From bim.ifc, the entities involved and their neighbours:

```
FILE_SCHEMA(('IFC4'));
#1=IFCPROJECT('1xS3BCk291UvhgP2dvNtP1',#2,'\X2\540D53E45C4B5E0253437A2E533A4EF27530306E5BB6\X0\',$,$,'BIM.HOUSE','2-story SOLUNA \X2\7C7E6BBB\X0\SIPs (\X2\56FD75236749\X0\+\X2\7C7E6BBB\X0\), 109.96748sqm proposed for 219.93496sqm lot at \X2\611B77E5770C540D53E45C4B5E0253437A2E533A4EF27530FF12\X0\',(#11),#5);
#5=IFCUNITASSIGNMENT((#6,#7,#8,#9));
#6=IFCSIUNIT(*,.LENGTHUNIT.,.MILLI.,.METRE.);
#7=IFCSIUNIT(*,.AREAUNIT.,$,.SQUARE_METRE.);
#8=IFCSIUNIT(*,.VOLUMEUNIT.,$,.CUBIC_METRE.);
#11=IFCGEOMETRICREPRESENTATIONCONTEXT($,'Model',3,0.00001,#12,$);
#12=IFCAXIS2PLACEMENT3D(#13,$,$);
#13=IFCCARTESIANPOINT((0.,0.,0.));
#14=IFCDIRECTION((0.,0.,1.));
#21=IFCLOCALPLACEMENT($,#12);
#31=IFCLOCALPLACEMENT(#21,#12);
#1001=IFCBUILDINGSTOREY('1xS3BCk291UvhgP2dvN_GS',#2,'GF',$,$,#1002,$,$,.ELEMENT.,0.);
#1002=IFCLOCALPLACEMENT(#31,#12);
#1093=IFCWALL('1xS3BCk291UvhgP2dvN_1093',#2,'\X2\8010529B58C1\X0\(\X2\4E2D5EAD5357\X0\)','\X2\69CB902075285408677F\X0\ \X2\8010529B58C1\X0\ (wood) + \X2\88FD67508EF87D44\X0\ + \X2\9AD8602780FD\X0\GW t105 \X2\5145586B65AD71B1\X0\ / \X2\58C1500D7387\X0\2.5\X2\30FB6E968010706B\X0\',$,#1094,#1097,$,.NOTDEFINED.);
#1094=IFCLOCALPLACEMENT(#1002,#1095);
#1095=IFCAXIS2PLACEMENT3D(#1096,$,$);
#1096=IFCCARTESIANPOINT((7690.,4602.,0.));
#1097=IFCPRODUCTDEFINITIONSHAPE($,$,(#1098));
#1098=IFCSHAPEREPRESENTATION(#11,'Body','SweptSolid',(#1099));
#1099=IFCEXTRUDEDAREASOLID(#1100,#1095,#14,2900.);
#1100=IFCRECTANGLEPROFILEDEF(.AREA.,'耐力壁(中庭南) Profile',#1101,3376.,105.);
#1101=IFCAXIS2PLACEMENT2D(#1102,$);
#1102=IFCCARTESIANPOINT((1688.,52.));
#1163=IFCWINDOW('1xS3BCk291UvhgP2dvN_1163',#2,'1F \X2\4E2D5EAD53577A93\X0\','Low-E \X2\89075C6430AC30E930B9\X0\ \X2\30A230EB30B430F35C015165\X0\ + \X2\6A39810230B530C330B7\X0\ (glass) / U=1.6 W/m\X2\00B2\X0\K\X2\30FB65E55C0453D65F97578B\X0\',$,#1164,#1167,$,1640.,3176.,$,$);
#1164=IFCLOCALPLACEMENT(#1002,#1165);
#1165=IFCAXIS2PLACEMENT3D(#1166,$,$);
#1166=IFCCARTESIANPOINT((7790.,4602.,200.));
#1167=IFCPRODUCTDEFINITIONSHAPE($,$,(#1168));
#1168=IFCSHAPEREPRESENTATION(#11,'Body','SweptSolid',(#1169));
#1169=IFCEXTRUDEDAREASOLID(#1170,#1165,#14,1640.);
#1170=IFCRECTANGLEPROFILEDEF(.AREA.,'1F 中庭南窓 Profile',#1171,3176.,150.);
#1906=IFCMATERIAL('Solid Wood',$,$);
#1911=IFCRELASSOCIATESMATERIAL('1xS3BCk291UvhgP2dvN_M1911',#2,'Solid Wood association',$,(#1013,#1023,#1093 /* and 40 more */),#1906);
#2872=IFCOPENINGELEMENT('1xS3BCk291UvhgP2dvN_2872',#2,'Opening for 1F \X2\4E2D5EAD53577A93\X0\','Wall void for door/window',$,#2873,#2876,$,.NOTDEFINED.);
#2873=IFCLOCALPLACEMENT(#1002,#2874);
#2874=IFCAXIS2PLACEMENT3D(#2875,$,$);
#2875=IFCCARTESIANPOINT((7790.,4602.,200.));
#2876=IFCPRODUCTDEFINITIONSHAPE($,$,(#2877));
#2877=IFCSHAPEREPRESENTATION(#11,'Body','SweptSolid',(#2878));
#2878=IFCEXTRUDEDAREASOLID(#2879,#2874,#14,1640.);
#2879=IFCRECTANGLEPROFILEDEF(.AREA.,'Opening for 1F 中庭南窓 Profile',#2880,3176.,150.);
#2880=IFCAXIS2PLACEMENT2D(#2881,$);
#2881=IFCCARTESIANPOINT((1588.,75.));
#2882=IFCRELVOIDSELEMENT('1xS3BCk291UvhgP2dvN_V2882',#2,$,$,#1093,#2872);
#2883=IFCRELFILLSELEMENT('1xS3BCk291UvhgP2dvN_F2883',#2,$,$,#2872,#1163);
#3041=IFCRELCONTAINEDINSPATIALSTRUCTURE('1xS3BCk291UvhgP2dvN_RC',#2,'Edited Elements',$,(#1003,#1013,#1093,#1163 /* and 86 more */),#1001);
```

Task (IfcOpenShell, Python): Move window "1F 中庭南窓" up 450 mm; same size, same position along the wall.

```python
import numpy as np
import ifcopenshell
import ifcopenshell.api.geometry
import ifcopenshell.util.placement
import ifcopenshell.util.unit

model = ifcopenshell.open("bim.ifc")
unit_scale = ifcopenshell.util.unit.calculate_unit_scale(model)

window = model.by_guid("1xS3BCk291UvhgP2dvN_1163")
opening = window.FillsVoids[0].RelatingOpeningElement
dz = 450.0

shift = np.array([0.0, 0.0, dz])
# The window is not placed relative to its opening, so move both.
for product in (opening, window):
    matrix = ifcopenshell.util.placement.get_local_placement(product.ObjectPlacement)
    matrix[:3, 3] += shift
    ifcopenshell.api.geometry.edit_object_placement(model, product=product, matrix=matrix, is_si=False)

print(f"moved by {dz * unit_scale:+.3f} m")

model.write("bim_rev.ifc")
```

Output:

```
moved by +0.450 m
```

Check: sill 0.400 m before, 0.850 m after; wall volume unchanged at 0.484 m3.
